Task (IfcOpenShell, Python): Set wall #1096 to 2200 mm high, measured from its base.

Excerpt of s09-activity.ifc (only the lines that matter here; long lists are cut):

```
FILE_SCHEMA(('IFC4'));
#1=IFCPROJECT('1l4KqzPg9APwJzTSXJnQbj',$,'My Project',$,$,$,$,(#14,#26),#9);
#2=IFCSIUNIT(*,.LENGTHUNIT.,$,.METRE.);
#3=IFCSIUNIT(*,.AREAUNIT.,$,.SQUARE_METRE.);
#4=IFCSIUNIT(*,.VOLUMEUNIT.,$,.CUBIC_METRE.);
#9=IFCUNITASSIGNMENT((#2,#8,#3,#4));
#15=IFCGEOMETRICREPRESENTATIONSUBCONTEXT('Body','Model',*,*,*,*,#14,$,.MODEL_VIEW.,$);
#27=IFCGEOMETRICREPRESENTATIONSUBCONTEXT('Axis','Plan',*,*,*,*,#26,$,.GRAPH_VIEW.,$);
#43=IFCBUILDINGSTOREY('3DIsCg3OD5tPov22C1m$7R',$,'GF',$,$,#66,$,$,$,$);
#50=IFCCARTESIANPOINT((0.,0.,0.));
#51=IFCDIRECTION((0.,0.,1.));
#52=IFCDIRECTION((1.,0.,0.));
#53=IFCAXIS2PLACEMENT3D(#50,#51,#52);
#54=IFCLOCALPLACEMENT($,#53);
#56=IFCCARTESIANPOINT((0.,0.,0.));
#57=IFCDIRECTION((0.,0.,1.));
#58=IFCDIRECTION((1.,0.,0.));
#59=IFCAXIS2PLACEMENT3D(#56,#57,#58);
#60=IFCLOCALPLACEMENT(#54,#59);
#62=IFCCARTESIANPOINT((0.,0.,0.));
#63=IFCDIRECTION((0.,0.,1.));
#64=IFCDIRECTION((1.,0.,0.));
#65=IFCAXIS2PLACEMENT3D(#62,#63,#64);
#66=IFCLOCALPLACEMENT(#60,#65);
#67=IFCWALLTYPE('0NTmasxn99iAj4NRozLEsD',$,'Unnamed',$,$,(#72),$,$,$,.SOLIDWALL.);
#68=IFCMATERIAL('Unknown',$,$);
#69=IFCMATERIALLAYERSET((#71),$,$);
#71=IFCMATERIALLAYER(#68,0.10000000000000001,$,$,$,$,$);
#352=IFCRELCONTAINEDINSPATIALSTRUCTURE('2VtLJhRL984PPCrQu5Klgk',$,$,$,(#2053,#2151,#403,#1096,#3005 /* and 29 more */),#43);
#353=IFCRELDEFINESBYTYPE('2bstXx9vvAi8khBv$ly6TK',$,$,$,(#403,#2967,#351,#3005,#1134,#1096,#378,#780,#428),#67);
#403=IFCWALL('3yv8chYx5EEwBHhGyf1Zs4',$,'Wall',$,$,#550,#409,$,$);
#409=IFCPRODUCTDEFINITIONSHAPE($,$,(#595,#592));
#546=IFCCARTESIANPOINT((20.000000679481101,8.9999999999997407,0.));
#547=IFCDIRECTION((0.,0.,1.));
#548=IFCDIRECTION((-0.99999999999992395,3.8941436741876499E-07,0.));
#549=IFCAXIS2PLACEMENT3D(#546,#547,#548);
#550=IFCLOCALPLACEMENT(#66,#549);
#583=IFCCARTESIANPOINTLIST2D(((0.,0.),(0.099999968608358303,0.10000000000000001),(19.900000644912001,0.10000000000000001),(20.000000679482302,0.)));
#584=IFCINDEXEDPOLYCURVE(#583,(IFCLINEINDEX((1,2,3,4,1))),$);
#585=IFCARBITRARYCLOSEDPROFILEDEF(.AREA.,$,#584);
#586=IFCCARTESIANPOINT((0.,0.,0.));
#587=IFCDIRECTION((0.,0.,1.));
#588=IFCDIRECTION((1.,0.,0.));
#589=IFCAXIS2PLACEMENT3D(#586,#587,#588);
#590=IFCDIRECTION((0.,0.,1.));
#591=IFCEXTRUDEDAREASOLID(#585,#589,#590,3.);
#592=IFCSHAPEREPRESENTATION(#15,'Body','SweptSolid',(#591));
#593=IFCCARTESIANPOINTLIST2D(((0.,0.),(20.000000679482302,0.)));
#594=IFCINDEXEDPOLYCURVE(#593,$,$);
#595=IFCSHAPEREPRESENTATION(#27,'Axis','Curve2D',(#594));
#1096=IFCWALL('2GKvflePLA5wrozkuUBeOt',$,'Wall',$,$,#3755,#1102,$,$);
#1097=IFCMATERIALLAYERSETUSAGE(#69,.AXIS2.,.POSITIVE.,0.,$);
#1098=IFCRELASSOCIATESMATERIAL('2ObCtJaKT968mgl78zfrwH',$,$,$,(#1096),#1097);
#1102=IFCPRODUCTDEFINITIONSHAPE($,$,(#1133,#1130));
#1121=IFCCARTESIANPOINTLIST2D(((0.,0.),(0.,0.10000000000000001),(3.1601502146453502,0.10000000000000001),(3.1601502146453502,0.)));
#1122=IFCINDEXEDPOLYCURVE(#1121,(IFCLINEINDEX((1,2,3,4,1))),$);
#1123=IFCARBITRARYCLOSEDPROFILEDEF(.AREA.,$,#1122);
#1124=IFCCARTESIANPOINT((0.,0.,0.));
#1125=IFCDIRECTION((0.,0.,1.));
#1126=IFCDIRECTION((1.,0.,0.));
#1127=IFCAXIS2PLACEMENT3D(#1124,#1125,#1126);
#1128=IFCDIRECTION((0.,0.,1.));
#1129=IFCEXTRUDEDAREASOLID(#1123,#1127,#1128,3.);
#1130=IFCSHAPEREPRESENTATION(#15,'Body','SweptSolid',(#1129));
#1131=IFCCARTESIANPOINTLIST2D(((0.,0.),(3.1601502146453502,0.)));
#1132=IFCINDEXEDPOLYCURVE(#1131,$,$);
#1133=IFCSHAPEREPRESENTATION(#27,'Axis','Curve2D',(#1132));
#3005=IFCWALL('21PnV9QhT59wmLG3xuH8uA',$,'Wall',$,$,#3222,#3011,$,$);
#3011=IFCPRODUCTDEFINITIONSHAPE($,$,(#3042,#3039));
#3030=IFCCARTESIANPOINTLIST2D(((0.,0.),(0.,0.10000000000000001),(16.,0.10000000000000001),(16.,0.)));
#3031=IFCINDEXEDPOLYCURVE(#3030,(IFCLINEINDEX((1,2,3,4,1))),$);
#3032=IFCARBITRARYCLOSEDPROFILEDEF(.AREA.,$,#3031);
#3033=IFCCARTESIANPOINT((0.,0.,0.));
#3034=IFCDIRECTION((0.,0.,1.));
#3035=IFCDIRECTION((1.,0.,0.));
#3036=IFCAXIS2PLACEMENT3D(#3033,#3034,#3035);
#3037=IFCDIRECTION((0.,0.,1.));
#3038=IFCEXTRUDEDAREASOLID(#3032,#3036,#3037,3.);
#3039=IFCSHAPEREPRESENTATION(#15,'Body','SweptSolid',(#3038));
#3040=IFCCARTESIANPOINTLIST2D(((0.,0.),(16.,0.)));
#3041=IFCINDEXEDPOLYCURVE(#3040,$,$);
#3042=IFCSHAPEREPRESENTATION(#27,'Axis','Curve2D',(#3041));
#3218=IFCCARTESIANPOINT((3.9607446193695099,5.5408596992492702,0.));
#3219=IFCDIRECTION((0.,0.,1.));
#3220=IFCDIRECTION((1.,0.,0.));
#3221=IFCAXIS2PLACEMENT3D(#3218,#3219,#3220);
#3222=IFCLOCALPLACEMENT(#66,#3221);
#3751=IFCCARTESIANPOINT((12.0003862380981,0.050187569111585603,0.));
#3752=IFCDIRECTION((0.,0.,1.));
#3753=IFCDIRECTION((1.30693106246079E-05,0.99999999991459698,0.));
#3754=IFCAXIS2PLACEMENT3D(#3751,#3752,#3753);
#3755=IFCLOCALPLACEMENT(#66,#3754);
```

```python
import ifcopenshell
import ifcopenshell.geom
import ifcopenshell.util.representation
import ifcopenshell.util.shape
import ifcopenshell.util.unit

model = ifcopenshell.open("s09-activity.ifc")
unit_scale = ifcopenshell.util.unit.calculate_unit_scale(model)
settings = ifcopenshell.geom.settings()


def volume(element):
    """Net volume in cubic metres, openings subtracted."""
    shape = ifcopenshell.geom.create_shape(settings, element)
    return ifcopenshell.util.shape.get_volume(shape.geometry)


wall = model.by_guid("2GKvflePLA5wrozkuUBeOt")
before = volume(wall)

body = ifcopenshell.util.representation.get_representation(wall, "Model", "Body")
solid = body.Items[0]
old_height = solid.Depth
solid.Depth = 2.2 / unit_scale
after = volume(wall)

print(f"height {old_height:g} -> {solid.Depth:g}, volume {before:.3f} -> {after:.3f} m3")

model.write("s09-activity_rev.ifc")
```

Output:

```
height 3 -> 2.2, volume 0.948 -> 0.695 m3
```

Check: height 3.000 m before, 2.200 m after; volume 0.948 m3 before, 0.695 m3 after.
